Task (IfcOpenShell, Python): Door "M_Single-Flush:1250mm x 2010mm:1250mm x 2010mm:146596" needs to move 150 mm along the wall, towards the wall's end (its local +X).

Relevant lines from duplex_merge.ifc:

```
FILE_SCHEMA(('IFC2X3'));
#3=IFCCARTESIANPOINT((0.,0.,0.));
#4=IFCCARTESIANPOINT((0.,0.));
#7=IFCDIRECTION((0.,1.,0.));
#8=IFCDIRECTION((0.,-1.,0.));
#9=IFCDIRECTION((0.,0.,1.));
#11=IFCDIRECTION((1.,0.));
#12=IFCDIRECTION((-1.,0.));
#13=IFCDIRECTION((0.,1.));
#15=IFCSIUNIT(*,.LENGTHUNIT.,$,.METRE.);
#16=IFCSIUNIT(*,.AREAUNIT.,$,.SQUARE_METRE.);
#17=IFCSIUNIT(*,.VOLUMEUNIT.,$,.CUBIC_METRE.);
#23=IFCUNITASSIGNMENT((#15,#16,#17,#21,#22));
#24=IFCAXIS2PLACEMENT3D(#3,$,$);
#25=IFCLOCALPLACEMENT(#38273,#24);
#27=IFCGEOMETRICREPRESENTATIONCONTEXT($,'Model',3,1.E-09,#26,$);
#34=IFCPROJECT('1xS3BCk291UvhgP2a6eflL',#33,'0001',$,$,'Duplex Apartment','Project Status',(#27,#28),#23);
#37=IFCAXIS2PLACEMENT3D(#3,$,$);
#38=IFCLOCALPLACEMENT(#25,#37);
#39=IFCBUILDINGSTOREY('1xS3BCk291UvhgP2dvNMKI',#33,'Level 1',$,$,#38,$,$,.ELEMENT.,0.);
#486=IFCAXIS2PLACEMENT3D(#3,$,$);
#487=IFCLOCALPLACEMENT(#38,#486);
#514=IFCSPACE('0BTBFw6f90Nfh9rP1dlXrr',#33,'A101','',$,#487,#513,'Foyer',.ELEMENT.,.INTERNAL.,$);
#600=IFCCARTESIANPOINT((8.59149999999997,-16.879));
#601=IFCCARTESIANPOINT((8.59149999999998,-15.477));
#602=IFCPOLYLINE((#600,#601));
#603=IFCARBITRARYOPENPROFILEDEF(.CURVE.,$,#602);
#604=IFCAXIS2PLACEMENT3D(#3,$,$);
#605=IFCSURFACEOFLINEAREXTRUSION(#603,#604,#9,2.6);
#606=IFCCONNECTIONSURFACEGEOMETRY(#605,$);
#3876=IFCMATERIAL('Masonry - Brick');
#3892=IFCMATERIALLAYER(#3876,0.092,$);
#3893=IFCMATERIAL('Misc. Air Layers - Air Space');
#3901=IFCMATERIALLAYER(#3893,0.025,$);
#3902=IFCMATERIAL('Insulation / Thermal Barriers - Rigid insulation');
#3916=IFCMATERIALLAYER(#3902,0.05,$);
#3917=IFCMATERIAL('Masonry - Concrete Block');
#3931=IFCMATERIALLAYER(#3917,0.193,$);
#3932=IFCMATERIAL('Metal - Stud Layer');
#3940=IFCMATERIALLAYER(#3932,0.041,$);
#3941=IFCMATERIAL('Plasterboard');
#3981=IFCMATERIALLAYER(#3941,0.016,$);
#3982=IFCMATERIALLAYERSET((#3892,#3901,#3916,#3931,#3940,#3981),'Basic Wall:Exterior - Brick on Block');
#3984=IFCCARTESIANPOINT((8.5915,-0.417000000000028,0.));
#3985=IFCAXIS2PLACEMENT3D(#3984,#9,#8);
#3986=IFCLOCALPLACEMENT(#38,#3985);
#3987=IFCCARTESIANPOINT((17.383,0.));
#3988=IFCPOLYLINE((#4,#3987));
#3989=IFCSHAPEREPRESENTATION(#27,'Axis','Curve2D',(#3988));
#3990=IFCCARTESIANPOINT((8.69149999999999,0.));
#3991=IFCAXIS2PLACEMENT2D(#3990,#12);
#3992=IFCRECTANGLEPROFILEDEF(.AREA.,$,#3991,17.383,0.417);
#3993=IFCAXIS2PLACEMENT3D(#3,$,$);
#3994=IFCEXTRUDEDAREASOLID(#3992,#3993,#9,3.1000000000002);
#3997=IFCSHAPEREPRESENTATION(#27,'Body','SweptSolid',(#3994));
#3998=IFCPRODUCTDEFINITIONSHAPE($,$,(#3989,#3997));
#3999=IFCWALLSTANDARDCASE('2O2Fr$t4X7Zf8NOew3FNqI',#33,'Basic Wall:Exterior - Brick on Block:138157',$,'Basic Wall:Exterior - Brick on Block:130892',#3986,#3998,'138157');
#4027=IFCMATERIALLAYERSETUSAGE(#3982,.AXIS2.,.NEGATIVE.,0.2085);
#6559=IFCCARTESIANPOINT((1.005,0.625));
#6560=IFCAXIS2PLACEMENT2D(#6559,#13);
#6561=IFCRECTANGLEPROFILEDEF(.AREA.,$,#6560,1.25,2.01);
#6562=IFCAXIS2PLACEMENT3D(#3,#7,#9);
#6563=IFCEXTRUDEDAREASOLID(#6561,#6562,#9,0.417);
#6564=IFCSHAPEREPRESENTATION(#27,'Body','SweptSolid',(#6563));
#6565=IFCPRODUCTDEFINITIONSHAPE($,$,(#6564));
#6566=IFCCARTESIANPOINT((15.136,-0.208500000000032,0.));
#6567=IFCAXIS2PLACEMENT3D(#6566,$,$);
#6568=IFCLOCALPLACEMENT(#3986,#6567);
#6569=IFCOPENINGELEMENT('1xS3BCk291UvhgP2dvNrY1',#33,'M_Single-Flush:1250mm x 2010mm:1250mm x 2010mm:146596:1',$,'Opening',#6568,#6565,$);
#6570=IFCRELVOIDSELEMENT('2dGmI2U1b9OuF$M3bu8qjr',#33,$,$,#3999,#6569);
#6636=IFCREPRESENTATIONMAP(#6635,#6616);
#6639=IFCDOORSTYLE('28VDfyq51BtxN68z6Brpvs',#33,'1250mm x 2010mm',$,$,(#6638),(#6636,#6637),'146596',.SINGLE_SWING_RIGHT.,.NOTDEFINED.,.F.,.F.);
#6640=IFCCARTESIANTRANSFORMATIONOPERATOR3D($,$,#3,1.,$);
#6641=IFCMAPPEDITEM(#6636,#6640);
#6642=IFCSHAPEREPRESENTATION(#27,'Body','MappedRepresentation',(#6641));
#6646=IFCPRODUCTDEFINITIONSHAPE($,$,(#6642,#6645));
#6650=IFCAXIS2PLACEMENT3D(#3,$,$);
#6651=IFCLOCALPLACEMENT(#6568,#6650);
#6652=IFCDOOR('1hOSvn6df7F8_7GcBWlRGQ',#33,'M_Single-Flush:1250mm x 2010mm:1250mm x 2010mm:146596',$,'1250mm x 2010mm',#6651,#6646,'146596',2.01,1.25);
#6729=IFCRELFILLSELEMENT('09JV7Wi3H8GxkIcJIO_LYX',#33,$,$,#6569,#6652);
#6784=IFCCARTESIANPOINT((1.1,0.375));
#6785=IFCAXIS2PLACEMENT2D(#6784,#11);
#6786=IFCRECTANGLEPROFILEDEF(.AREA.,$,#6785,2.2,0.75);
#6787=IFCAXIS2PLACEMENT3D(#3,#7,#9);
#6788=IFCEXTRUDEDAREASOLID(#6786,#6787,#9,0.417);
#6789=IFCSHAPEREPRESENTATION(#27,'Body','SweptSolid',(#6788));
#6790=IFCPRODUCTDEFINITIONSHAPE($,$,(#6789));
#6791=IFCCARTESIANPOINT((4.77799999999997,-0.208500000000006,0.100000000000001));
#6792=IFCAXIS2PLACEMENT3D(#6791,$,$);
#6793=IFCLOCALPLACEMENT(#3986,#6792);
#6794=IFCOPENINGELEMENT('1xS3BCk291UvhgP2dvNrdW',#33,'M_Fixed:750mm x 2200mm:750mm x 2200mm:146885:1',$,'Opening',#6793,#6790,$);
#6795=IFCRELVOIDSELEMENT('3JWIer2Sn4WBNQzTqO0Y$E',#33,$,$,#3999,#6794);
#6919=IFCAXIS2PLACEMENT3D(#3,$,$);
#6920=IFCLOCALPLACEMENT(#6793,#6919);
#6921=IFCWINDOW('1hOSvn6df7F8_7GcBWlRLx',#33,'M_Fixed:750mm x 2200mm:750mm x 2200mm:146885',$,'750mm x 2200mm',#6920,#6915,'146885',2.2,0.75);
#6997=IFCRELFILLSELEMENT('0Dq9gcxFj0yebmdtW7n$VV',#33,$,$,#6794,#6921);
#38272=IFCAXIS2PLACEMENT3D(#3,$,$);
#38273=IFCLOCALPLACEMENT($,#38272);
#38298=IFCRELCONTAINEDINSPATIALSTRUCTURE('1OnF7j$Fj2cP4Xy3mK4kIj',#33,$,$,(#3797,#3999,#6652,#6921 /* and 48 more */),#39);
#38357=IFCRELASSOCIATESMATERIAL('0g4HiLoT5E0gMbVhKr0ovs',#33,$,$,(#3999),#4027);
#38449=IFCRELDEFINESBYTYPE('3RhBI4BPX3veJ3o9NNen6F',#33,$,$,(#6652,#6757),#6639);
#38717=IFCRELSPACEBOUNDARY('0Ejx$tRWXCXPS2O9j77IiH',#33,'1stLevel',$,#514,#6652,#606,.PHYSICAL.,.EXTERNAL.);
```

```python
import numpy as np
import ifcopenshell
import ifcopenshell.api.geometry
import ifcopenshell.util.placement

model = ifcopenshell.open("duplex_merge.ifc")

door = model.by_guid("1hOSvn6df7F8_7GcBWlRGQ")
opening = door.FillsVoids[0].RelatingOpeningElement
wall = opening.VoidsElements[0].RelatingBuildingElement

wall_matrix = ifcopenshell.util.placement.get_local_placement(wall.ObjectPlacement)
shift = wall_matrix[:3, 0] * 0.15
before = ifcopenshell.util.placement.get_local_placement(door.ObjectPlacement)[:3, 3].copy()

# The door is placed relative to its opening, so it follows when the opening moves.
matrix = ifcopenshell.util.placement.get_local_placement(opening.ObjectPlacement)
matrix[:3, 3] += shift
ifcopenshell.api.geometry.edit_object_placement(
    model, product=opening, matrix=matrix, is_si=False, should_transform_children=True
)

# Space boundary surfaces are stored in each space's coordinates; move them too.
for rel in door.ProvidesBoundaries:
    if not rel.ConnectionGeometry:
        continue
    surface = rel.ConnectionGeometry.SurfaceOnRelatingElement
    space_matrix = ifcopenshell.util.placement.get_local_placement(rel.RelatingSpace.ObjectPlacement)
    point = np.array(surface.Position.Location.Coordinates) + space_matrix[:3, :3].T @ shift
    surface.Position = model.createIfcAxis2Placement3D(
        model.createIfcCartesianPoint(point.tolist()), surface.Position.Axis, surface.Position.RefDirection
    )

after = ifcopenshell.util.placement.get_local_placement(door.ObjectPlacement)[:3, 3]
print("door moved by", (after - before).round(3) + 0.0)

model.write("duplex_merge-out.ifc")
```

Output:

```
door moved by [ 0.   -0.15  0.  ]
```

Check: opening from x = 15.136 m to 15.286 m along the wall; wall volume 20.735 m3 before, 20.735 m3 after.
